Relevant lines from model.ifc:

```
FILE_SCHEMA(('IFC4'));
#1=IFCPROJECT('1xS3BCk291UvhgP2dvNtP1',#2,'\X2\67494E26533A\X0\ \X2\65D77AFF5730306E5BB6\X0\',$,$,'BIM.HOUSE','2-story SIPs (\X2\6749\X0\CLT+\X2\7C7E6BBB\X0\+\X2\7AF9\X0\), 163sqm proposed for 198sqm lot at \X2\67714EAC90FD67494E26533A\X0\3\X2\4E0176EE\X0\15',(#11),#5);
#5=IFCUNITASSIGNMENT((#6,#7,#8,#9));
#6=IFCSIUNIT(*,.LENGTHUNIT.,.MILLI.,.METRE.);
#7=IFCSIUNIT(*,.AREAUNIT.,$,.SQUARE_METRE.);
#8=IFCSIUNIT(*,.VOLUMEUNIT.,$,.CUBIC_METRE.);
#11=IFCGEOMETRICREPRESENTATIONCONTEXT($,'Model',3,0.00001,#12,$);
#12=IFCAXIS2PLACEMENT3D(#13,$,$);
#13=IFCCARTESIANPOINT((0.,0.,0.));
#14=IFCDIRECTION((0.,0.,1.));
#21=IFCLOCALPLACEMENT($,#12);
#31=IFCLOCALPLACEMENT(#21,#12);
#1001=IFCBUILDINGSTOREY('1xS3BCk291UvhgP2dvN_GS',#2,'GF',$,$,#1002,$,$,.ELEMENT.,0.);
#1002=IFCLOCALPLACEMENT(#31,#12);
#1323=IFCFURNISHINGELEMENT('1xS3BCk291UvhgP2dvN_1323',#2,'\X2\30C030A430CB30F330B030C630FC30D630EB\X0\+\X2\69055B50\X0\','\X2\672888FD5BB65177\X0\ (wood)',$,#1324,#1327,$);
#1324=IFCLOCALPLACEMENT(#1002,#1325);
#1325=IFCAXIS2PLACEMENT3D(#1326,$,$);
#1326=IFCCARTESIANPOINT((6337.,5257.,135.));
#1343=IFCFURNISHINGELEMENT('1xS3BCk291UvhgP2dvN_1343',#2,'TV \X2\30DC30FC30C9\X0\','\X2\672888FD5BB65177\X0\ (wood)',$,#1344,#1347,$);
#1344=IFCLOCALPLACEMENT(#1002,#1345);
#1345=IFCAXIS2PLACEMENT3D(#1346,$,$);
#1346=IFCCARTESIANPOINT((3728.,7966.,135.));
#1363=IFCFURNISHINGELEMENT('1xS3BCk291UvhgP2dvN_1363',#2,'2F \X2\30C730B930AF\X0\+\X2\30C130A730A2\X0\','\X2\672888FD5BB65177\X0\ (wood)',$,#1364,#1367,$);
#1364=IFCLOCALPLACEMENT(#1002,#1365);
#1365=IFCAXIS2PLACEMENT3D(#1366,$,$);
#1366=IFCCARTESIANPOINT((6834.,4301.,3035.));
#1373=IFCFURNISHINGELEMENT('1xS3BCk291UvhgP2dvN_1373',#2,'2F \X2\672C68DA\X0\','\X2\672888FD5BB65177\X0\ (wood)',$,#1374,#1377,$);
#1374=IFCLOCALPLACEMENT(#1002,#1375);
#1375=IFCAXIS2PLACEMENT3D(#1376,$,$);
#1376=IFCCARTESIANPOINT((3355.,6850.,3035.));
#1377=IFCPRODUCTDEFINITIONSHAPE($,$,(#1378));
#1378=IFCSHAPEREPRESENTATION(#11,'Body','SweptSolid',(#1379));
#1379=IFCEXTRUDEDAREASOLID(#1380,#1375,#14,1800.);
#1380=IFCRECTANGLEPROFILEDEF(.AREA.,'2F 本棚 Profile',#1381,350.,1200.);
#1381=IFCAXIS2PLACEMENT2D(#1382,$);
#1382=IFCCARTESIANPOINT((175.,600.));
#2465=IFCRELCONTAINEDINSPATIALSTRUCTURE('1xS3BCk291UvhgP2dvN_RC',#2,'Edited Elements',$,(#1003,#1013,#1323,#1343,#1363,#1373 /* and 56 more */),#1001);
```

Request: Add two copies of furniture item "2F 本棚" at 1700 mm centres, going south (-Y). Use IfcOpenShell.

```python
import numpy as np
import ifcopenshell
import ifcopenshell.api.geometry
import ifcopenshell.api.root
import ifcopenshell.util.element
import ifcopenshell.util.placement

model = ifcopenshell.open("model.ifc")


def reuse_history(source, copy):
    """copy_class also copies each property set's owner history, people and application; keep the originals."""
    for rel in copy.IsDefinedBy:
        if rel.is_a("IfcRelDefinesByProperties") and (history := rel.RelatingPropertyDefinition.OwnerHistory):
            rel.RelatingPropertyDefinition.OwnerHistory = source.OwnerHistory
            ifcopenshell.util.element.remove_deep2(model, history)


source = model.by_guid("1xS3BCk291UvhgP2dvN_1373")
base = ifcopenshell.util.placement.get_local_placement(source.ObjectPlacement)
step = np.array([0.0, -1.0, 0.0]) * 1700.0

for i in range(1, 3):
    copy = ifcopenshell.api.root.copy_class(model, product=source)
    copy.Representation = ifcopenshell.util.element.copy_deep(
        model, source.Representation, exclude=["IfcGeometricRepresentationContext", "IfcRepresentationMap"]
    )
    reuse_history(source, copy)
    matrix = base.copy()
    matrix[:3, 3] += i * step
    print("added at", matrix[:3, 3].round(3) + 0.0)
    ifcopenshell.api.geometry.edit_object_placement(model, product=copy, matrix=matrix, is_si=False)

model.write("model_rev.ifc")
```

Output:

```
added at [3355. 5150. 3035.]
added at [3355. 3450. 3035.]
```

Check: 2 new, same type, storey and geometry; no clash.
